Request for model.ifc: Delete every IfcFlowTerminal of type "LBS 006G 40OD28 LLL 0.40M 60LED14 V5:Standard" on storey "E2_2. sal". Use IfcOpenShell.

First a look at what the model holds.

```python
import ifcopenshell
import ifcopenshell.util.element

model = ifcopenshell.open("model.ifc")
print(model.schema)
storey = next(s for s in model.by_type("IfcBuildingStorey") if s.Name == "E2_2. sal")
terminals = [e for e in ifcopenshell.util.element.get_decomposition(storey) if e.is_a("IfcFlowTerminal")]
seen = {}
for e in terminals:
    element_type = ifcopenshell.util.element.get_type(e)
    name = element_type.Name if element_type not in (None, e) else None
    seen[name] = seen.get(name, 0) + 1
for name, count in sorted(seen.items(), key=str):
    print(count, "x", name)
```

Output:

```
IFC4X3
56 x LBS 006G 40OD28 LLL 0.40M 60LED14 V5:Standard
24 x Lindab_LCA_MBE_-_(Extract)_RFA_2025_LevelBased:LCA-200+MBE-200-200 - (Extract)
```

```python
import ifcopenshell
import ifcopenshell.api.root
import ifcopenshell.util.element

model = ifcopenshell.open("model.ifc")

storey = next(s for s in model.by_type("IfcBuildingStorey") if s.Name == "E2_2. sal")
terminals = [e for e in ifcopenshell.util.element.get_decomposition(storey) if e.is_a("IfcFlowTerminal")]
targets = [e for e in terminals if (t := ifcopenshell.util.element.get_type(e)) not in (None, e) and t.Name == "LBS 006G 40OD28 LLL 0.40M 60LED14 V5:Standard"]

for e in targets:
    ifcopenshell.api.root.remove_product(model, product=e)
print(len(targets), "removed")

model.write("model_edited.ifc")
```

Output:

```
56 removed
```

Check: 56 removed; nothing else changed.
